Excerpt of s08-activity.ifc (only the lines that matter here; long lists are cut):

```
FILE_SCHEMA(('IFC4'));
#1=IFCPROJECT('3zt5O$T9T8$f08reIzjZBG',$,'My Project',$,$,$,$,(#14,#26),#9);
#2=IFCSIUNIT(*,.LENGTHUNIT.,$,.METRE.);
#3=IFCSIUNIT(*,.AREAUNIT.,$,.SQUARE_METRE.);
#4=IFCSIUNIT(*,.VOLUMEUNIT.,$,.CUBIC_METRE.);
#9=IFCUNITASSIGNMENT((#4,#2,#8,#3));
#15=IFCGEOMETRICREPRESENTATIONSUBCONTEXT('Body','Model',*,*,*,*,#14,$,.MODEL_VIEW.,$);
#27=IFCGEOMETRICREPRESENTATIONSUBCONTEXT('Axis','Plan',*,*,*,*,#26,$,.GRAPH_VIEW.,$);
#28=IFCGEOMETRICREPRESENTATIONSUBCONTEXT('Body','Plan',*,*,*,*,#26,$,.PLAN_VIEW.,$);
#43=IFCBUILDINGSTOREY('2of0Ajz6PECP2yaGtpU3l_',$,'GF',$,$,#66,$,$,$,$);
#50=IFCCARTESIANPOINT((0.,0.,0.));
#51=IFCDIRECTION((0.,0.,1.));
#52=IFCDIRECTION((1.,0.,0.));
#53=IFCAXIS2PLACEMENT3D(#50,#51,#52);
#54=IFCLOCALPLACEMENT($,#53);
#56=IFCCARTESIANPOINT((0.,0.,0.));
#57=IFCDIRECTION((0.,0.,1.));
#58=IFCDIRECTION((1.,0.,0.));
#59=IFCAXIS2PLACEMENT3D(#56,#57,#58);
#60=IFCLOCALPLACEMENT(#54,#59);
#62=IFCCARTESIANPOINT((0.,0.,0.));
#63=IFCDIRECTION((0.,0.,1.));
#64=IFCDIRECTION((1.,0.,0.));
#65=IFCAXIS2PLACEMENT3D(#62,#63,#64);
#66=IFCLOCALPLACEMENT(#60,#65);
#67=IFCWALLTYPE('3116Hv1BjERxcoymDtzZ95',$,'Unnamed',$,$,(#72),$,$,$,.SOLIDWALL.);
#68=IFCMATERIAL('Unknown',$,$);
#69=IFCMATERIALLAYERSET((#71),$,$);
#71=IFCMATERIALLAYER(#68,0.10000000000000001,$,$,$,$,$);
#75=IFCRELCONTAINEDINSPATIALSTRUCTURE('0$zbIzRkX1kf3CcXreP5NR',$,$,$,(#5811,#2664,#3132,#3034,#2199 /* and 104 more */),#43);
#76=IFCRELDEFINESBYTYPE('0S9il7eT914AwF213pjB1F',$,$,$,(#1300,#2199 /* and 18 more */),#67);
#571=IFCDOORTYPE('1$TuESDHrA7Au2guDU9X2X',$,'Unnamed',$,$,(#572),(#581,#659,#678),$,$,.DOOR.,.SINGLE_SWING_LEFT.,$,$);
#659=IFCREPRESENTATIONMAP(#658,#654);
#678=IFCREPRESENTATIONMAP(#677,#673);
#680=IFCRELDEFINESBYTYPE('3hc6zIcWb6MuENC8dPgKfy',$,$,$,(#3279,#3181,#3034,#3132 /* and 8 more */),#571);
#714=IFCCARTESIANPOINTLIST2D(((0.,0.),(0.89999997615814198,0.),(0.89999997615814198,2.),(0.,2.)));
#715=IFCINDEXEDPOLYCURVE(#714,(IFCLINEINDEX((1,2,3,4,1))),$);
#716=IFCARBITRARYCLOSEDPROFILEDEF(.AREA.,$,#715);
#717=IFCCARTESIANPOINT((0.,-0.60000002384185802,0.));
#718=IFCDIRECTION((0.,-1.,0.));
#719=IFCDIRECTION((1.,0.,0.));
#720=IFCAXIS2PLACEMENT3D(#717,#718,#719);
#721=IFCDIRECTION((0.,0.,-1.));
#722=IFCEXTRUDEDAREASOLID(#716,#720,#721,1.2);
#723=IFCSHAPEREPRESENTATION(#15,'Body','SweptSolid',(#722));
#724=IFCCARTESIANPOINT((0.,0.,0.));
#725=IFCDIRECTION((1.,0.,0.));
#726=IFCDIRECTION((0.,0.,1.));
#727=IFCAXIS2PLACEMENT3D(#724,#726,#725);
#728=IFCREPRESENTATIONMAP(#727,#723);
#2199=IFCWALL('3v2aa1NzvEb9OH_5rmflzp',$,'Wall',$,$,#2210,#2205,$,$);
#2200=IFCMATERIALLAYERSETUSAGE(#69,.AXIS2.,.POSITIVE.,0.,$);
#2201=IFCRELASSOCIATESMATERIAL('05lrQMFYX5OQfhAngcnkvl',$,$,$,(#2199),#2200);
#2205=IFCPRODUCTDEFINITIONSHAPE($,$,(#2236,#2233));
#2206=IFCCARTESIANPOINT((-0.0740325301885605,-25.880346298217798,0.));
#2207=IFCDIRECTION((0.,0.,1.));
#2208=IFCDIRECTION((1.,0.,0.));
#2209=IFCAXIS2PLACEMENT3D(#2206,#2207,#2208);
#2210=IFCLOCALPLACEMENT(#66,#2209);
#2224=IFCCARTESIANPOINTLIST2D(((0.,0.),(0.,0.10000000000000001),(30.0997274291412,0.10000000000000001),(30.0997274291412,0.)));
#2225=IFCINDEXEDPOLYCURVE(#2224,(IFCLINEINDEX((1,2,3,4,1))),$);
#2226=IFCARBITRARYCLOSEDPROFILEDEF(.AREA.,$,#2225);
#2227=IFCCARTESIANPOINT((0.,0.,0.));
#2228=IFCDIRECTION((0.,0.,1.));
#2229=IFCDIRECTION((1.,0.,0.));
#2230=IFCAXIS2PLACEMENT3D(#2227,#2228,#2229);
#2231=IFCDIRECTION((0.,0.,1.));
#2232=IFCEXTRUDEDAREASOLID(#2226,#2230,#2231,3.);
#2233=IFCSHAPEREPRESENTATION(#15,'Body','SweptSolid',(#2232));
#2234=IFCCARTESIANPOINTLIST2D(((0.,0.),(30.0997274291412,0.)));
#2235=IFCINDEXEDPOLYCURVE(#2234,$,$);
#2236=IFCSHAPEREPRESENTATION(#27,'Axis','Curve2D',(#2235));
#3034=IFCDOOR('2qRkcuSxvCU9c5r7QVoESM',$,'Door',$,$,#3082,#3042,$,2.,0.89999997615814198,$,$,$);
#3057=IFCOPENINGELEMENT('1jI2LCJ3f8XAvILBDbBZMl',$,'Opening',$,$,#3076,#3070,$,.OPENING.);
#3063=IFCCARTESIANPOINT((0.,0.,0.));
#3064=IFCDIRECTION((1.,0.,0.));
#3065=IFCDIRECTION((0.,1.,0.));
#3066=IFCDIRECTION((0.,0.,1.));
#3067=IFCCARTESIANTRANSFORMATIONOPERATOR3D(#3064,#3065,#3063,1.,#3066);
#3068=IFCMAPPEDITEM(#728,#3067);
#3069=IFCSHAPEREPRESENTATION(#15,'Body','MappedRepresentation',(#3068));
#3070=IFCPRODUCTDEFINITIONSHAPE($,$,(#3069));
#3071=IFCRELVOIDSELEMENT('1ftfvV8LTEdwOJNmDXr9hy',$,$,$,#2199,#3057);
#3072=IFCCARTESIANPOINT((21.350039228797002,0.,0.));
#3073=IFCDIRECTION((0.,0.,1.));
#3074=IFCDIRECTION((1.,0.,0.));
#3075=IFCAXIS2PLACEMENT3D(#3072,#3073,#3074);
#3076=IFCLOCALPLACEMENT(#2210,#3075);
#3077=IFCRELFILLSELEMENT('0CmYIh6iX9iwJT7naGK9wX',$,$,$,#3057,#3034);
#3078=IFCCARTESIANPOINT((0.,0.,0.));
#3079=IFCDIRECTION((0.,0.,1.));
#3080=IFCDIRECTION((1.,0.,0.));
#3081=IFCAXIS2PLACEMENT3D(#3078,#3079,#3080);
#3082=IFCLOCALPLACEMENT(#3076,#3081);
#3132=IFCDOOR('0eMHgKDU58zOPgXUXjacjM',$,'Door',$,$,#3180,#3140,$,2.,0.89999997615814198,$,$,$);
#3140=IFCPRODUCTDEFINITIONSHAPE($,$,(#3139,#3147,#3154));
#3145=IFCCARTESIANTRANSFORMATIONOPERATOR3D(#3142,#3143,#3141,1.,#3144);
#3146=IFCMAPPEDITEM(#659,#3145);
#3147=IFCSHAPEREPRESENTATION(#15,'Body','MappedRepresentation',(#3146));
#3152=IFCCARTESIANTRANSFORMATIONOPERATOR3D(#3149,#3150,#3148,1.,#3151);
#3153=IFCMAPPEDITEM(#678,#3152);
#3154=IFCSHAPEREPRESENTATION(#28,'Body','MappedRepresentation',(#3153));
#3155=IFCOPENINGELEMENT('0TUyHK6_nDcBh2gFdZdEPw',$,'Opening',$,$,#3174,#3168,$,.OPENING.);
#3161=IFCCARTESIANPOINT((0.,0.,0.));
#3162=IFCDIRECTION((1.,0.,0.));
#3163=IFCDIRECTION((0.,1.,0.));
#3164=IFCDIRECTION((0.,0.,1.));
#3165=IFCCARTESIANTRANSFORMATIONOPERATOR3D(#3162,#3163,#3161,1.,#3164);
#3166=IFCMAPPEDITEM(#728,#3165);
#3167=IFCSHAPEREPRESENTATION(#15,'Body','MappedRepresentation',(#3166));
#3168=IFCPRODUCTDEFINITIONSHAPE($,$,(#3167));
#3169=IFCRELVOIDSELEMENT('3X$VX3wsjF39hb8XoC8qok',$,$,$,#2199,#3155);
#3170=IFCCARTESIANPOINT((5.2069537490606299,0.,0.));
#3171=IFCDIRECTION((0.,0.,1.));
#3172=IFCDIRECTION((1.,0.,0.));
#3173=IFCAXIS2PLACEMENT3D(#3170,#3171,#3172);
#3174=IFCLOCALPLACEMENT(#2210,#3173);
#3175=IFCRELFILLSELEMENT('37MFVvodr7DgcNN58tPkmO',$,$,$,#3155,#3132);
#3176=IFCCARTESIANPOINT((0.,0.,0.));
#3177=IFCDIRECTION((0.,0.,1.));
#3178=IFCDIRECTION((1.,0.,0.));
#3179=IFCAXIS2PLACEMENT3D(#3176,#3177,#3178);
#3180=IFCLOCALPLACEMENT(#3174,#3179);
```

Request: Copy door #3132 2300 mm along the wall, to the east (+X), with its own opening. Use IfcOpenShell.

```python
import ifcopenshell
import ifcopenshell.api.feature
import ifcopenshell.api.geometry
import ifcopenshell.api.root
import ifcopenshell.geom
import ifcopenshell.util.element
import ifcopenshell.util.placement
import ifcopenshell.util.shape

model = ifcopenshell.open("s08-activity.ifc")
settings = ifcopenshell.geom.settings()


def volume(element):
    """Net volume in cubic metres, openings subtracted."""
    shape = ifcopenshell.geom.create_shape(settings, element)
    return ifcopenshell.util.shape.get_volume(shape.geometry)


door = model.by_id(3132)
opening = door.FillsVoids[0].RelatingOpeningElement
wall = opening.VoidsElements[0].RelatingBuildingElement
before = volume(wall)
shift = ifcopenshell.util.placement.get_local_placement(wall.ObjectPlacement)[:3, 0] * 2.3

# copy_class copies the void relationship, type, container and properties, but no geometry.
new_opening = ifcopenshell.api.root.copy_class(model, product=opening)
new_opening.Representation = ifcopenshell.util.element.copy_deep(
    model, opening.Representation, exclude=["IfcGeometricRepresentationContext", "IfcRepresentationMap"]
)
new_door = ifcopenshell.api.root.copy_class(model, product=door)
new_door.Representation = ifcopenshell.util.element.copy_deep(
    model, door.Representation, exclude=["IfcGeometricRepresentationContext", "IfcRepresentationMap"]
)
ifcopenshell.api.feature.add_filling(model, opening=new_opening, element=new_door)

for old, new in ((opening, new_opening), (door, new_door)):
    matrix = ifcopenshell.util.placement.get_local_placement(old.ObjectPlacement)
    matrix[:3, 3] += shift
    ifcopenshell.api.geometry.edit_object_placement(model, product=new, matrix=matrix, is_si=False)

after = volume(wall)

print(f"wall volume {before:.3f} -> {after:.3f} m3")

model.write("s08-activity_edited.ifc")
```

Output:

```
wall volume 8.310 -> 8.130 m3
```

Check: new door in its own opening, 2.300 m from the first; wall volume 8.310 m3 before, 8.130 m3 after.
